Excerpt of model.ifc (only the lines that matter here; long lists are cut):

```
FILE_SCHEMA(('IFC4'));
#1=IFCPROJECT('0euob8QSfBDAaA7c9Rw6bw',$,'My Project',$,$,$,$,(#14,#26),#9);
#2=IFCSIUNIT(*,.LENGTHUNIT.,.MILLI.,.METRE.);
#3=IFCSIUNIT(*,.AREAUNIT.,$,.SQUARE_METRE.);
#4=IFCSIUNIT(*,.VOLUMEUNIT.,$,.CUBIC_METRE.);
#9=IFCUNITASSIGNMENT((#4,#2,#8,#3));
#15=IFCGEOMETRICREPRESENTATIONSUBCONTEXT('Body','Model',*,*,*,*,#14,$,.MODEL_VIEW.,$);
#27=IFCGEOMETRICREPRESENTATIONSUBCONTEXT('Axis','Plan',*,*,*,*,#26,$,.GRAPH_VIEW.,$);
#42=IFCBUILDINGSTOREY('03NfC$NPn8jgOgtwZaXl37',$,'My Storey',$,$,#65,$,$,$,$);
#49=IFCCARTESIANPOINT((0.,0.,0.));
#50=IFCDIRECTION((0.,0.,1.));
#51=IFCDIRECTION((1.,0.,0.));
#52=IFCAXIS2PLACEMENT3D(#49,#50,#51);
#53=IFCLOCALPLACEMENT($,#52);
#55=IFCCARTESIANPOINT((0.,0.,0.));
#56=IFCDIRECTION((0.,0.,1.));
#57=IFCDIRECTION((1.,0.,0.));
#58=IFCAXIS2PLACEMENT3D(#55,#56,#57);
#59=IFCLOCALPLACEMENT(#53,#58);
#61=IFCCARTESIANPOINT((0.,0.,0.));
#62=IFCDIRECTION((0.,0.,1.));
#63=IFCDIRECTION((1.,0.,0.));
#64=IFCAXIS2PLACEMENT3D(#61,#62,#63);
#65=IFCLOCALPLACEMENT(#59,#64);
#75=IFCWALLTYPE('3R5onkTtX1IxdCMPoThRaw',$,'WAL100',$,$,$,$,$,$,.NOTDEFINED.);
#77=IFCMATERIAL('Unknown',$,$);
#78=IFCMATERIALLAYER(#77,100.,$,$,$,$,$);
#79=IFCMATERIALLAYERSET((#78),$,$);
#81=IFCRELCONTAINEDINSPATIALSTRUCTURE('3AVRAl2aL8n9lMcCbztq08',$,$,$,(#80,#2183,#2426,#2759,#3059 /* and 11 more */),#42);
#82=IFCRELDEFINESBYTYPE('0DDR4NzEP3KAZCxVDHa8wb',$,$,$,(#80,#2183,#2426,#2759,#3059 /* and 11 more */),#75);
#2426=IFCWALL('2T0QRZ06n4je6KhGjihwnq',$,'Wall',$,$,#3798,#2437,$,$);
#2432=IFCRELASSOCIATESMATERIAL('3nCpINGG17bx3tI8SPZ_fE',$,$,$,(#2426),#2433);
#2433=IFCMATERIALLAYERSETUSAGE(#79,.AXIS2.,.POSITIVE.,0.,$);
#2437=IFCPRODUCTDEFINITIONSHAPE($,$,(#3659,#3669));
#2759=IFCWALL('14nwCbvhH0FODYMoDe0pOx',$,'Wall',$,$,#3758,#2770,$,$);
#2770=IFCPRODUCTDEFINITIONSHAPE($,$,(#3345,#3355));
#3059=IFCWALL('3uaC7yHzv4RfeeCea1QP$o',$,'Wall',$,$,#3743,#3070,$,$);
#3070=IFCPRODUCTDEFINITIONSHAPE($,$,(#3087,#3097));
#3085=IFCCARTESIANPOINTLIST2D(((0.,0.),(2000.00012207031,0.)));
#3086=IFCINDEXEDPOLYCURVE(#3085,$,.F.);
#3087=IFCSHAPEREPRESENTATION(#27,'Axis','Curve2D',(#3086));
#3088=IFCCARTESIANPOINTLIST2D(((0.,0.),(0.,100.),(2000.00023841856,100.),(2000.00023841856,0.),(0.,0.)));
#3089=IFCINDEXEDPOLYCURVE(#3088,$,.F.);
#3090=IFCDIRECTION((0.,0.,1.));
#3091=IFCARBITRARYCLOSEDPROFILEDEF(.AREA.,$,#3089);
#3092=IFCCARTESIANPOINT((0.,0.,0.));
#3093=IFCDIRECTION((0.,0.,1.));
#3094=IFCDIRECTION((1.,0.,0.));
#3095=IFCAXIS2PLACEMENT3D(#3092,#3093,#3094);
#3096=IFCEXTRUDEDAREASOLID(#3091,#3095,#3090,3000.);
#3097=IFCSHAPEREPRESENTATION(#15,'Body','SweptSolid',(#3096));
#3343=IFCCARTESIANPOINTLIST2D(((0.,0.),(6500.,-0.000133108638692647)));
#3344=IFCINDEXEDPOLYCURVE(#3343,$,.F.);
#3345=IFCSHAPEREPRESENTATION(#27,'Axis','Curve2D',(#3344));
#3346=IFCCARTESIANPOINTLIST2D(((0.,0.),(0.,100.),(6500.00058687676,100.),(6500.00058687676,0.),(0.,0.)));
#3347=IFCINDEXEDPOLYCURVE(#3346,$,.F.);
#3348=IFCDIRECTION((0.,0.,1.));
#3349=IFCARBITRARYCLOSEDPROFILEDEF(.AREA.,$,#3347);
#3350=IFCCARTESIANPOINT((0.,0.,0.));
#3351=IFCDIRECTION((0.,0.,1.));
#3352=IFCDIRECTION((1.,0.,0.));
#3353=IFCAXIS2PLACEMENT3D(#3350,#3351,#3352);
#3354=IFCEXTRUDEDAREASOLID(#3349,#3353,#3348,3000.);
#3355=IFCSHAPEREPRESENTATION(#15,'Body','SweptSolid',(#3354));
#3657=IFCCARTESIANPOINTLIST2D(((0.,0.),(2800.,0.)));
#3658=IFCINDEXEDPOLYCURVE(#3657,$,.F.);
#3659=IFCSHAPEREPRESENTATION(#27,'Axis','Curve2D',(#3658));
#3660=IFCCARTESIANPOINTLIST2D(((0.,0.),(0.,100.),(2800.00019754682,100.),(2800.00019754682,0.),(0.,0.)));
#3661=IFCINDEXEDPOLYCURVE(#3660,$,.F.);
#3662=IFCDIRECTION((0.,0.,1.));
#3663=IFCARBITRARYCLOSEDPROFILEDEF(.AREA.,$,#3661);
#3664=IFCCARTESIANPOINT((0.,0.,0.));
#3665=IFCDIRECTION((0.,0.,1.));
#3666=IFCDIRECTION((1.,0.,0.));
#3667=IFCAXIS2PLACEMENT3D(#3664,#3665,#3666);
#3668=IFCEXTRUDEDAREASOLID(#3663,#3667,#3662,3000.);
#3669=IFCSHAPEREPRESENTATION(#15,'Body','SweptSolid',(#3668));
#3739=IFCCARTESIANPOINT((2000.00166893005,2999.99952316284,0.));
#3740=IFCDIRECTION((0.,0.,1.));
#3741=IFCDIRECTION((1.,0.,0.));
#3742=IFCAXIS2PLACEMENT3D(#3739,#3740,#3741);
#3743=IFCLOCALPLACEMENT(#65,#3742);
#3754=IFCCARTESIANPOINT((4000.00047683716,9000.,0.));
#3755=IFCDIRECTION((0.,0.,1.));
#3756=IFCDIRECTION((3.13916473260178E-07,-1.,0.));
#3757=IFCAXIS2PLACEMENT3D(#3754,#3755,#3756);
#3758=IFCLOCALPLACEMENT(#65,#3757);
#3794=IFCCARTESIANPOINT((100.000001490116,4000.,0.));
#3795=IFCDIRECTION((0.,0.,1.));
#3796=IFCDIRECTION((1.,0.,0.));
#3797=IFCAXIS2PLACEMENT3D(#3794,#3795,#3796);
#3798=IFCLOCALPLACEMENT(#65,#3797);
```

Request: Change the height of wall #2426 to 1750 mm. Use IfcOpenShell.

```python
import ifcopenshell
import ifcopenshell.geom
import ifcopenshell.util.representation
import ifcopenshell.util.shape
import ifcopenshell.util.unit

model = ifcopenshell.open("model.ifc")
unit_scale = ifcopenshell.util.unit.calculate_unit_scale(model)
settings = ifcopenshell.geom.settings()


def volume(element):
    """Net volume in cubic metres, openings subtracted."""
    shape = ifcopenshell.geom.create_shape(settings, element)
    return ifcopenshell.util.shape.get_volume(shape.geometry)


wall = model.by_id(2426)
before = volume(wall)

body = ifcopenshell.util.representation.get_representation(wall, "Model", "Body")
solid = body.Items[0]
old_height = solid.Depth
solid.Depth = 1.75 / unit_scale
after = volume(wall)

print(f"height {old_height:g} -> {solid.Depth:g}, volume {before:.3f} -> {after:.3f} m3")

model.write("model_v2.ifc")
```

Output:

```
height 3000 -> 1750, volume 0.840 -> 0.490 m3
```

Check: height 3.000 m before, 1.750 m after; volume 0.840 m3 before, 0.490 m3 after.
